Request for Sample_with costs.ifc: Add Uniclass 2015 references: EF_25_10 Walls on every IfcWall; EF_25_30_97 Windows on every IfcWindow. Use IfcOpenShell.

First a look at what the model holds.

```python
import ifcopenshell

model = ifcopenshell.open("Sample_with costs.ifc")
print(model.schema)
print("classifications:", [c.Name for c in model.by_type("IfcClassification")])
for ifc_class in ("IfcDoor", "IfcRoof", "IfcStair", "IfcWall", "IfcWindow"):
    print(ifc_class, len(model.by_type(ifc_class)))
```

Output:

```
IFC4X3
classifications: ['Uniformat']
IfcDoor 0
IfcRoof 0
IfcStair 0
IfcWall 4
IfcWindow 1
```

```python
import ifcopenshell
import ifcopenshell.api.classification

model = ifcopenshell.open("Sample_with costs.ifc")

system = ifcopenshell.api.classification.add_classification(model, classification="Uniclass 2015")

codes = {
    "IfcWall": ("EF_25_10", "Walls"),
    "IfcWindow": ("EF_25_30_97", "Windows"),
}
for ifc_class, (code, name) in codes.items():
    products = model.by_type(ifc_class)
    ifcopenshell.api.classification.add_reference(
        model, products=products, classification=system, identification=code, name=name
    )
    print(code, len(products))

model.write("Sample_with costs_edited.ifc")
```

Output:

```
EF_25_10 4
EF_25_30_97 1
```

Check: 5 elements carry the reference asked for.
